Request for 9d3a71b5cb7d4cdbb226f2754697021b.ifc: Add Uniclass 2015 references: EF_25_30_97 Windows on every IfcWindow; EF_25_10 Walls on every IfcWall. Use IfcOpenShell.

First a look at what the model holds.

```python
import ifcopenshell

model = ifcopenshell.open("9d3a71b5cb7d4cdbb226f2754697021b.ifc")
print(model.schema)
print("classifications:", [c.Name for c in model.by_type("IfcClassification")])
for ifc_class in ("IfcDoor", "IfcRoof", "IfcStair", "IfcWall", "IfcWindow"):
    print(ifc_class, len(model.by_type(ifc_class)))
```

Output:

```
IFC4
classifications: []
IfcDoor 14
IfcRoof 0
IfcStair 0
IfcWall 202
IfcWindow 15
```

```python
import ifcopenshell
import ifcopenshell.api.classification

model = ifcopenshell.open("9d3a71b5cb7d4cdbb226f2754697021b.ifc")

system = ifcopenshell.api.classification.add_classification(model, classification="Uniclass 2015")

codes = {
    "IfcWindow": ("EF_25_30_97", "Windows"),
    "IfcWall": ("EF_25_10", "Walls"),
}
for ifc_class, (code, name) in codes.items():
    products = model.by_type(ifc_class)
    ifcopenshell.api.classification.add_reference(
        model, products=products, classification=system, identification=code, name=name
    )
    print(code, len(products))

model.write("9d3a71b5cb7d4cdbb226f2754697021b_edited.ifc")
```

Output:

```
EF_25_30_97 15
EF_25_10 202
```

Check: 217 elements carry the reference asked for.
